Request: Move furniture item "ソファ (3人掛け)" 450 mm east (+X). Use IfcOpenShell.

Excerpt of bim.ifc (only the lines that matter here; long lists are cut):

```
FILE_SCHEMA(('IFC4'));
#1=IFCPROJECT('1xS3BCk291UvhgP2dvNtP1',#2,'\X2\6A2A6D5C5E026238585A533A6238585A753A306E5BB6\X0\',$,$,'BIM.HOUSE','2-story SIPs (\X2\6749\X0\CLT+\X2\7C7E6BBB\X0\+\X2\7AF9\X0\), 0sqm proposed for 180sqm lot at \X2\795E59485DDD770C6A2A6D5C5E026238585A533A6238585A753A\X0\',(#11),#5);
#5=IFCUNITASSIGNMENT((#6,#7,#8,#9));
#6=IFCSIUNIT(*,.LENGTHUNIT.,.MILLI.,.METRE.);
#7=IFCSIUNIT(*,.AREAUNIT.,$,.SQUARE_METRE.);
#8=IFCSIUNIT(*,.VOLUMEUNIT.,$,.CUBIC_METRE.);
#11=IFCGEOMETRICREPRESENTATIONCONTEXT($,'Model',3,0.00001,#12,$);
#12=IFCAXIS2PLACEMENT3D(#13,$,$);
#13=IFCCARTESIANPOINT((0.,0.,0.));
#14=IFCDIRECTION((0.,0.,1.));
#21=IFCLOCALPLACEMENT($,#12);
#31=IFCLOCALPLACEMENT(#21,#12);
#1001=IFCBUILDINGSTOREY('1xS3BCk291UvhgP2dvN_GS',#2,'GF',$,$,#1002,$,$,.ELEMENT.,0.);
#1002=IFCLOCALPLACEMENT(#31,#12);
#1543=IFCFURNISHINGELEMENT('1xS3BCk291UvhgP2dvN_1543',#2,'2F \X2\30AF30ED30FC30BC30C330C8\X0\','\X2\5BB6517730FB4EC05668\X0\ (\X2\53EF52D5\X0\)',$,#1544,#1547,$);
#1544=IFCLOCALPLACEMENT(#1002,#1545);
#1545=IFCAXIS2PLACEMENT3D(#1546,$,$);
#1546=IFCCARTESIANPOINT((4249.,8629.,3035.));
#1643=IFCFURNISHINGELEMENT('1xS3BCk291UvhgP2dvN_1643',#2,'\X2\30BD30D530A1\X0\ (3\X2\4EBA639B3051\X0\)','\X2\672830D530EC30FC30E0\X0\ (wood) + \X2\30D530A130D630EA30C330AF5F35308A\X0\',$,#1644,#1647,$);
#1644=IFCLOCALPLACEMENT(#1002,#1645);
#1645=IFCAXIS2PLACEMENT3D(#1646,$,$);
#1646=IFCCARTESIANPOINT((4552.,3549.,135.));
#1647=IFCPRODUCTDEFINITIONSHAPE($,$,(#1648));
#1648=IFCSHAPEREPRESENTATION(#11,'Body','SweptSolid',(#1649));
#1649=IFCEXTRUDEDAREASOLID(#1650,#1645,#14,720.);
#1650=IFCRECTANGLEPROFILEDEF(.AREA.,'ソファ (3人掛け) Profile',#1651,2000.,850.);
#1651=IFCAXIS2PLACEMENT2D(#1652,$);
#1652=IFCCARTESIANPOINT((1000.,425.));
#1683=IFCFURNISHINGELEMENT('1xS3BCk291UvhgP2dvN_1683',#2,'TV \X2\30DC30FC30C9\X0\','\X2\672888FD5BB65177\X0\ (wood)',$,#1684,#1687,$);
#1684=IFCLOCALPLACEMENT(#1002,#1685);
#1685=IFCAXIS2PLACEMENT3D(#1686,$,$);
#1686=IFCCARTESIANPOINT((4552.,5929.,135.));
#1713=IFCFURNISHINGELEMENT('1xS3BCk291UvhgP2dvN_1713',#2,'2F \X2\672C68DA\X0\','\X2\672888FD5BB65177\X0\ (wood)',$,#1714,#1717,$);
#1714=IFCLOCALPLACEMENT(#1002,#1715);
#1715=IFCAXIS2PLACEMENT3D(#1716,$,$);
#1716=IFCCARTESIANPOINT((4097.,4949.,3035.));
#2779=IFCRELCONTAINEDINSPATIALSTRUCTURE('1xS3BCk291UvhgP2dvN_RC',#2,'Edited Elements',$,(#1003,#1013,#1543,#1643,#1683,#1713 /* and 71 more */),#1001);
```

```python
import ifcopenshell
import ifcopenshell.api.geometry
import ifcopenshell.util.placement
import ifcopenshell.util.unit

model = ifcopenshell.open("bim.ifc")
unit_scale = ifcopenshell.util.unit.calculate_unit_scale(model)

item = model.by_guid("1xS3BCk291UvhgP2dvN_1643")
matrix = ifcopenshell.util.placement.get_local_placement(item.ObjectPlacement)
matrix[0, 3] += 0.45 / unit_scale
ifcopenshell.api.geometry.edit_object_placement(model, product=item, matrix=matrix, is_si=False)

print(ifcopenshell.util.placement.get_local_placement(item.ObjectPlacement).round(3) + 0.0)

model.write("bim_edited.ifc")
```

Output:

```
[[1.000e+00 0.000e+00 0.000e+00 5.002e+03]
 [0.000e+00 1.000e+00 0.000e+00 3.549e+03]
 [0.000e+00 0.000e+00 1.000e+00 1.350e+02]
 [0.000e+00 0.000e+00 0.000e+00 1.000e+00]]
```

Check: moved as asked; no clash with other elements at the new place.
